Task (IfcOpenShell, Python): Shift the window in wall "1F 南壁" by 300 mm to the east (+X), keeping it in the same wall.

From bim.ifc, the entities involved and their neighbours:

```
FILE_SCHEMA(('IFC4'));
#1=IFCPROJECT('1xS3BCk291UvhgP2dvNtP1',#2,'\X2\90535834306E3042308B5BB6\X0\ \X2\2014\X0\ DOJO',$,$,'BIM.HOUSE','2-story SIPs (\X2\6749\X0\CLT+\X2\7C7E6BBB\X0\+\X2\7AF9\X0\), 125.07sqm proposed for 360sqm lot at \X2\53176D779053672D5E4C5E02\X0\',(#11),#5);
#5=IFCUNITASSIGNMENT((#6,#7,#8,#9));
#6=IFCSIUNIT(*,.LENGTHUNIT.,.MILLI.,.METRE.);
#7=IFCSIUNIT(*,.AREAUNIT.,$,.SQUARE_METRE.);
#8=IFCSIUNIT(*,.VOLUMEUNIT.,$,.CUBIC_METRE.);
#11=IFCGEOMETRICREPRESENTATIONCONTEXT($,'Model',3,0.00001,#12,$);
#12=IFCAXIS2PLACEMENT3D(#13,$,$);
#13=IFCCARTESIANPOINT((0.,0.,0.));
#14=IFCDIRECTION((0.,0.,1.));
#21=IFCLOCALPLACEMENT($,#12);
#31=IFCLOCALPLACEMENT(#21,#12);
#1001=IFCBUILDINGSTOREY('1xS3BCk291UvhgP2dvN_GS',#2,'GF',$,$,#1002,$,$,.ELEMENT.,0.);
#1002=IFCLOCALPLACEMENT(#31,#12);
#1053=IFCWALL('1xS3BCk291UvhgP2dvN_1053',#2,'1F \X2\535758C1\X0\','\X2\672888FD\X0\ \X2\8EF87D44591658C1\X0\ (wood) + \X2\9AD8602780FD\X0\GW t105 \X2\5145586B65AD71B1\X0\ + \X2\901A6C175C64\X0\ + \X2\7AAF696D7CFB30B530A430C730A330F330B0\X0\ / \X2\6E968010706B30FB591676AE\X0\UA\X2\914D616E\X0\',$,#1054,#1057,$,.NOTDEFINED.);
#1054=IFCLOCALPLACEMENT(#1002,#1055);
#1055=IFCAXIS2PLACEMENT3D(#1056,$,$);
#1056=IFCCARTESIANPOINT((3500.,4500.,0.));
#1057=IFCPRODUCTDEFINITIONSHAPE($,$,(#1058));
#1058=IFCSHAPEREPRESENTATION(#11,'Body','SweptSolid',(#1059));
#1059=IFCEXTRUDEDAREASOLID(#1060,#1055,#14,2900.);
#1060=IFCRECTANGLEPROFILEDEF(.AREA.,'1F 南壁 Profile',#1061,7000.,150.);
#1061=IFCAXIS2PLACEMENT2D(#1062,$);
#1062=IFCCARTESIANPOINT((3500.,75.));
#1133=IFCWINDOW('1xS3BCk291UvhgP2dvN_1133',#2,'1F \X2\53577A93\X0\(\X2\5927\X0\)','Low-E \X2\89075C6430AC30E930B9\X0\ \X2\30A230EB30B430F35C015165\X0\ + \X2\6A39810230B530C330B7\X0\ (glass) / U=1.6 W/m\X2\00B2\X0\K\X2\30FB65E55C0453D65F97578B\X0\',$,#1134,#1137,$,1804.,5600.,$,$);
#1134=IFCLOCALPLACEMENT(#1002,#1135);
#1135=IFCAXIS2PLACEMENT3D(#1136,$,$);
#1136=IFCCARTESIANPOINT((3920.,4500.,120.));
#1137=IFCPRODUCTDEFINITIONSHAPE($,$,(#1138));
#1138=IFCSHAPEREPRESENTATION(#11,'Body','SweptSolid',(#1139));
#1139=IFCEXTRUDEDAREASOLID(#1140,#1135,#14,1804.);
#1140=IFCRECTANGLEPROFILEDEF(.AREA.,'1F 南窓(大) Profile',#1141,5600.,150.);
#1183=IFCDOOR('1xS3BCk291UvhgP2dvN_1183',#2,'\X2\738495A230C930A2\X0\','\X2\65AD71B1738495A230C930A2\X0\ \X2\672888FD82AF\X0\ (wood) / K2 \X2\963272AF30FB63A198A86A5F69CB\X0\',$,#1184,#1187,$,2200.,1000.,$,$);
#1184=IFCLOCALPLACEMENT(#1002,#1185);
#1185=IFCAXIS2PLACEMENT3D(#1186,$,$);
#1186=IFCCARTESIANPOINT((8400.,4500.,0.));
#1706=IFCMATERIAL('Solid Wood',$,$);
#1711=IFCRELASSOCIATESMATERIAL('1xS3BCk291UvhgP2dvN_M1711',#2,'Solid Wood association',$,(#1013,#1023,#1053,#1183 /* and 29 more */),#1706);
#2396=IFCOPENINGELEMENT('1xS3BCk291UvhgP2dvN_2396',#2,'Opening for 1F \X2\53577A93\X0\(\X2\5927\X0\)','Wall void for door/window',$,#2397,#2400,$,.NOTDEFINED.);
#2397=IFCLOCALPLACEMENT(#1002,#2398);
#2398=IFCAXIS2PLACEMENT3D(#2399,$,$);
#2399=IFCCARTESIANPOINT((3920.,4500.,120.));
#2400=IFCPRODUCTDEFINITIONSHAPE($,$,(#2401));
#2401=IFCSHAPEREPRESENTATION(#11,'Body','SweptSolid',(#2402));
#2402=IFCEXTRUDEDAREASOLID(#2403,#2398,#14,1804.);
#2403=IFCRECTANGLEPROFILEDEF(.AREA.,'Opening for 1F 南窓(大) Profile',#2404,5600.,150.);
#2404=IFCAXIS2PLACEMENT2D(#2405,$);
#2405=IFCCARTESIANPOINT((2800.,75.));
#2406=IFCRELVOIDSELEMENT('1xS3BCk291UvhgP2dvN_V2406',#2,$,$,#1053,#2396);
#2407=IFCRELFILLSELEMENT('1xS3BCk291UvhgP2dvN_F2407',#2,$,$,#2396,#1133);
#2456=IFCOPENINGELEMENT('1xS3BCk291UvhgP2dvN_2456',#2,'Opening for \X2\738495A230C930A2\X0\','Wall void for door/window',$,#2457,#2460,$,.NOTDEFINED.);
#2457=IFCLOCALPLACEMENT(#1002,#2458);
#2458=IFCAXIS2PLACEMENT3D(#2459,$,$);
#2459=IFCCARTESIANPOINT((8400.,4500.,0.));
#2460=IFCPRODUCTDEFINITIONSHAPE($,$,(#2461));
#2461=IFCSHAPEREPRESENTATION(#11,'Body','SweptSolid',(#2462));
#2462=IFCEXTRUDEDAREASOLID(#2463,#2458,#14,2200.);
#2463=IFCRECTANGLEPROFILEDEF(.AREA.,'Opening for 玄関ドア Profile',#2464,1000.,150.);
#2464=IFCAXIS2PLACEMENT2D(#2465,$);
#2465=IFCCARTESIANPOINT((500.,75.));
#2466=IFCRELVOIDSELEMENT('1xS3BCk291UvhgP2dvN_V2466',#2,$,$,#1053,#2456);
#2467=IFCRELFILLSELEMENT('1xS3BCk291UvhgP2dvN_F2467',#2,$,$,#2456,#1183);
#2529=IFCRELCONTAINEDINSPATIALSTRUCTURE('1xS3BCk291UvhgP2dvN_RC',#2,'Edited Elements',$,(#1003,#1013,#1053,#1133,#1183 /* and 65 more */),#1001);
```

```python
import ifcopenshell
import ifcopenshell.api.geometry
import ifcopenshell.util.placement
import ifcopenshell.util.unit

model = ifcopenshell.open("bim.ifc")
unit_scale = ifcopenshell.util.unit.calculate_unit_scale(model)

window = model.by_guid("1xS3BCk291UvhgP2dvN_1133")
opening = window.FillsVoids[0].RelatingOpeningElement
wall = opening.VoidsElements[0].RelatingBuildingElement

wall_matrix = ifcopenshell.util.placement.get_local_placement(wall.ObjectPlacement)
shift = wall_matrix[:3, 0] * 0.3 / unit_scale
before = ifcopenshell.util.placement.get_local_placement(window.ObjectPlacement)[:3, 3].copy()

# The window is not placed relative to its opening, so move both.
for product in (opening, window):
    matrix = ifcopenshell.util.placement.get_local_placement(product.ObjectPlacement)
    matrix[:3, 3] += shift
    ifcopenshell.api.geometry.edit_object_placement(model, product=product, matrix=matrix, is_si=False)

after = ifcopenshell.util.placement.get_local_placement(window.ObjectPlacement)[:3, 3]
print("window moved by", (after - before).round(3) + 0.0)

model.write("bim_rev.ifc")
```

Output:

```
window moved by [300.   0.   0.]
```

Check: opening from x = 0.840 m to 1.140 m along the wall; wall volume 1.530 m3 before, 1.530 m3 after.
